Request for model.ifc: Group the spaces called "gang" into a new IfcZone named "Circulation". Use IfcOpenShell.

First a look at what the model holds.

```python
import ifcopenshell

model = ifcopenshell.open("model.ifc")
print(model.schema)
seen = {}
for space in model.by_type("IfcSpace"):
    seen[space.LongName] = seen.get(space.LongName, 0) + 1
for name, count in sorted(seen.items(), key=str):
    print(count, "x", name)
print("zones:", [z.Name for z in model.by_type("IfcZone")][:20])
```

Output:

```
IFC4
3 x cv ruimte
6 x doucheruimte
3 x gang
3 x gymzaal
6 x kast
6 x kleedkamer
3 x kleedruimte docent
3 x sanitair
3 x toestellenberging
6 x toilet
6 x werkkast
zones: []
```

```python
import ifcopenshell
import ifcopenshell.api.group
import ifcopenshell.api.root

model = ifcopenshell.open("model.ifc")

names = {"gang"}
spaces = [s for s in model.by_type("IfcSpace") if s.LongName in names]

zone = ifcopenshell.api.root.create_entity(model, ifc_class="IfcZone", name="Circulation")
ifcopenshell.api.group.assign_group(model, products=spaces, group=zone)
print(len(spaces), "spaces in", zone.Name)

model.write("model_rev.ifc")
```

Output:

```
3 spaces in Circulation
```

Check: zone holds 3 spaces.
